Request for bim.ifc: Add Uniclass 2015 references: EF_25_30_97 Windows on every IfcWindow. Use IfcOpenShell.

First a look at what the model holds.

```python
import ifcopenshell

model = ifcopenshell.open("bim.ifc")
print(model.schema)
print("classifications:", [c.Name for c in model.by_type("IfcClassification")])
for ifc_class in ("IfcDoor", "IfcRoof", "IfcStair", "IfcWall", "IfcWindow"):
    print(ifc_class, len(model.by_type(ifc_class)))
```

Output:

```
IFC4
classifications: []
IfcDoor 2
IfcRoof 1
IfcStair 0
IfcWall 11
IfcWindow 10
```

```python
import ifcopenshell
import ifcopenshell.api.classification

model = ifcopenshell.open("bim.ifc")

system = ifcopenshell.api.classification.add_classification(model, classification="Uniclass 2015")

codes = {
    "IfcWindow": ("EF_25_30_97", "Windows"),
}
for ifc_class, (code, name) in codes.items():
    products = model.by_type(ifc_class)
    ifcopenshell.api.classification.add_reference(
        model, products=products, classification=system, identification=code, name=name
    )
    print(code, len(products))

model.write("bim_edited.ifc")
```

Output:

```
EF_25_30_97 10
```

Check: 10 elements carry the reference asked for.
